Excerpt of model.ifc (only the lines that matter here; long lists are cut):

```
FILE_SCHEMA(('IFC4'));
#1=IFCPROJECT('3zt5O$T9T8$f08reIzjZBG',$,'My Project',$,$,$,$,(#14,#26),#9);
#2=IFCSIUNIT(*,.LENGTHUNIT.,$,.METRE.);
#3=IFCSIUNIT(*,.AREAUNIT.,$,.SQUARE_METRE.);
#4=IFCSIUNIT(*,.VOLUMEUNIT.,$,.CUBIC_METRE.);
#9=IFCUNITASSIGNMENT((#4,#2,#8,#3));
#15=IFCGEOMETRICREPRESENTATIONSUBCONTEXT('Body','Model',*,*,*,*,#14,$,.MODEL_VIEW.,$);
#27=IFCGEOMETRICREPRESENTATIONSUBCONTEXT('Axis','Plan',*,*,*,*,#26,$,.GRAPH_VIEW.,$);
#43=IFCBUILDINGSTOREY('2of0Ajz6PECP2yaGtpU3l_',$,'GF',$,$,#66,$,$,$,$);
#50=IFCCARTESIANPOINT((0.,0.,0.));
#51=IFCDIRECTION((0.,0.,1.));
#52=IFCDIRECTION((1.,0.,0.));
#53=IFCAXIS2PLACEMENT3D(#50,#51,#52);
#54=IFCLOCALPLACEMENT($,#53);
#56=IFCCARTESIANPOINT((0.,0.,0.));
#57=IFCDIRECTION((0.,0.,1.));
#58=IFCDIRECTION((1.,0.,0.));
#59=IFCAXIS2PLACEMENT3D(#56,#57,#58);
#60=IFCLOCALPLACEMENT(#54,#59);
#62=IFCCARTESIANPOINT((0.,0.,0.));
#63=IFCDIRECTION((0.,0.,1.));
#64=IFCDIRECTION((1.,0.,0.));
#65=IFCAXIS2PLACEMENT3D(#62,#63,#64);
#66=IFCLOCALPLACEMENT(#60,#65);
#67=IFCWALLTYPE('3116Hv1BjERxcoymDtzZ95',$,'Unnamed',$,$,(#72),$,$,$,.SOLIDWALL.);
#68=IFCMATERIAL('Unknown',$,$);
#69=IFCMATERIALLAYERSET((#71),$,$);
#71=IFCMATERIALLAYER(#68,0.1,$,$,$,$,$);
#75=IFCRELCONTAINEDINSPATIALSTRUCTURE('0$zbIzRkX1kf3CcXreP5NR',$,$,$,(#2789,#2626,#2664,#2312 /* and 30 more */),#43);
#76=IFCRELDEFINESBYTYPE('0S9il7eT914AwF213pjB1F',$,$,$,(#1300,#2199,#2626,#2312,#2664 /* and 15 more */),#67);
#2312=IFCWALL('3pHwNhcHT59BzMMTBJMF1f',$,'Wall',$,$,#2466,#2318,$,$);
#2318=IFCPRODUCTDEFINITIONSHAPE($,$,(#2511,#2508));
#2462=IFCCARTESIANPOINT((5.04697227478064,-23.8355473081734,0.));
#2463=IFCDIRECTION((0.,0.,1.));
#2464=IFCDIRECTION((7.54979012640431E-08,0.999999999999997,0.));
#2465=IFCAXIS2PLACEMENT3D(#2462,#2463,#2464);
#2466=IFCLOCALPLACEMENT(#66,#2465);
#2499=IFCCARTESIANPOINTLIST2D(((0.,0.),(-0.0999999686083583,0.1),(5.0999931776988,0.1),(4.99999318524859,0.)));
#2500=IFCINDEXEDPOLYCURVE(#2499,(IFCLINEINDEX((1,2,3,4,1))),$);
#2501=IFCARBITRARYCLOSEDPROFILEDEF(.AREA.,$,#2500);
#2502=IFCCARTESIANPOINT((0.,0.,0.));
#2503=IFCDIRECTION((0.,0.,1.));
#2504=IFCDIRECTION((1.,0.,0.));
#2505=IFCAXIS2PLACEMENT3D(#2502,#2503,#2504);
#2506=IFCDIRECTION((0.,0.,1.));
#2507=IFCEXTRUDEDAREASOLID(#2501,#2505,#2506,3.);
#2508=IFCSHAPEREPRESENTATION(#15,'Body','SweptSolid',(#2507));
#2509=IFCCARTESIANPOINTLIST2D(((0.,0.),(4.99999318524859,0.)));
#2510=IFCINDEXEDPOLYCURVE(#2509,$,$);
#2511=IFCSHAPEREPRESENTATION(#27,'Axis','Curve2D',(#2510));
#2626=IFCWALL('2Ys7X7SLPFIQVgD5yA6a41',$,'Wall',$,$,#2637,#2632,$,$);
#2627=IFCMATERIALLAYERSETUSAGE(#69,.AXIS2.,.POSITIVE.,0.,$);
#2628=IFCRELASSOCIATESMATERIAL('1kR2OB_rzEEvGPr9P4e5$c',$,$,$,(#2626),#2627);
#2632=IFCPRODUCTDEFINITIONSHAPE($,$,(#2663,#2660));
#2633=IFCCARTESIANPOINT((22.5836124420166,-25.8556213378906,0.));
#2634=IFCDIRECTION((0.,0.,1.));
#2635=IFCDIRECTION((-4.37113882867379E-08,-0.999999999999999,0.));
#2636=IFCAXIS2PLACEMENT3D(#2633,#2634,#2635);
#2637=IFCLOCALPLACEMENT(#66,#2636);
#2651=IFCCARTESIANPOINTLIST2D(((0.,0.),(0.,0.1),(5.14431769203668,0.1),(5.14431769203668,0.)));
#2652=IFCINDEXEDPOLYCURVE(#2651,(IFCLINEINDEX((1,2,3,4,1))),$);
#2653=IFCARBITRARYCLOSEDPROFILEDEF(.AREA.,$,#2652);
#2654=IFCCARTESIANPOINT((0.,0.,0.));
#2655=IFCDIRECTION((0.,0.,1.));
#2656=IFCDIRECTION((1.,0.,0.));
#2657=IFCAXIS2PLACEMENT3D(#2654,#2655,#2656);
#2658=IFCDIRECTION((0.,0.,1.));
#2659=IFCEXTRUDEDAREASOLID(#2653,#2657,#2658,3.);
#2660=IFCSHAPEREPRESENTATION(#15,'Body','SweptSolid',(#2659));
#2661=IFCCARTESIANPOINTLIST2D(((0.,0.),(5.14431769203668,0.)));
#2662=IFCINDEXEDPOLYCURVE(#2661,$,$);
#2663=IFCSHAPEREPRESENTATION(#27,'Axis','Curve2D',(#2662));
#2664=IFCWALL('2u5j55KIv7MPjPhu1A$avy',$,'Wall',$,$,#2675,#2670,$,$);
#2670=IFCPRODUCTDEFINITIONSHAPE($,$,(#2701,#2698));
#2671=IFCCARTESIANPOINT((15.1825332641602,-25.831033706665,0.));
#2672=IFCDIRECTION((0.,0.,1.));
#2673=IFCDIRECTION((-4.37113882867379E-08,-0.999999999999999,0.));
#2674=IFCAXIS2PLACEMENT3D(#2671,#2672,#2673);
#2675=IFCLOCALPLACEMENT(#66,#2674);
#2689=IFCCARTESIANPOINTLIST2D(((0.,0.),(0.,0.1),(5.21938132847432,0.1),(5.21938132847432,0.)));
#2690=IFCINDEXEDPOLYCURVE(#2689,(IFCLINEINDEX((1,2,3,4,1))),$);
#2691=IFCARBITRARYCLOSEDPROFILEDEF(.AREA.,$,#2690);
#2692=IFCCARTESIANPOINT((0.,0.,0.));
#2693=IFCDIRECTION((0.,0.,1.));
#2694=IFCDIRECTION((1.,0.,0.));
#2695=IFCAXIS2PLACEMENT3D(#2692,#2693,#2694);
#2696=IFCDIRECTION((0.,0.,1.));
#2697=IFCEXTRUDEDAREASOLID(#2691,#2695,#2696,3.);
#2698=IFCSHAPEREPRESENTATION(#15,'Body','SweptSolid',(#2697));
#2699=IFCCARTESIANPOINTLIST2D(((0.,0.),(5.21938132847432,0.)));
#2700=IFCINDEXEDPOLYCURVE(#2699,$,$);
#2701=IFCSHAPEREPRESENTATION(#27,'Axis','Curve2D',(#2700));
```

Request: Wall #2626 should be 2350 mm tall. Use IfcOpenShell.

```python
import ifcopenshell
import ifcopenshell.geom
import ifcopenshell.util.representation
import ifcopenshell.util.shape

model = ifcopenshell.open("model.ifc")
settings = ifcopenshell.geom.settings()


def volume(element):
    """Net volume in cubic metres, openings subtracted."""
    shape = ifcopenshell.geom.create_shape(settings, element)
    return ifcopenshell.util.shape.get_volume(shape.geometry)


wall = model.by_guid("2Ys7X7SLPFIQVgD5yA6a41")
before = volume(wall)

body = ifcopenshell.util.representation.get_representation(wall, "Model", "Body")
solid = body.Items[0]
old_height = solid.Depth
solid.Depth = 2.35
after = volume(wall)

print(f"height {old_height:g} -> {solid.Depth:g}, volume {before:.3f} -> {after:.3f} m3")

model.write("model_v2.ifc")
```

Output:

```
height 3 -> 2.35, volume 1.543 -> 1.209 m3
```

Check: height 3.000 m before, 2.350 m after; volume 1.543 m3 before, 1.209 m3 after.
